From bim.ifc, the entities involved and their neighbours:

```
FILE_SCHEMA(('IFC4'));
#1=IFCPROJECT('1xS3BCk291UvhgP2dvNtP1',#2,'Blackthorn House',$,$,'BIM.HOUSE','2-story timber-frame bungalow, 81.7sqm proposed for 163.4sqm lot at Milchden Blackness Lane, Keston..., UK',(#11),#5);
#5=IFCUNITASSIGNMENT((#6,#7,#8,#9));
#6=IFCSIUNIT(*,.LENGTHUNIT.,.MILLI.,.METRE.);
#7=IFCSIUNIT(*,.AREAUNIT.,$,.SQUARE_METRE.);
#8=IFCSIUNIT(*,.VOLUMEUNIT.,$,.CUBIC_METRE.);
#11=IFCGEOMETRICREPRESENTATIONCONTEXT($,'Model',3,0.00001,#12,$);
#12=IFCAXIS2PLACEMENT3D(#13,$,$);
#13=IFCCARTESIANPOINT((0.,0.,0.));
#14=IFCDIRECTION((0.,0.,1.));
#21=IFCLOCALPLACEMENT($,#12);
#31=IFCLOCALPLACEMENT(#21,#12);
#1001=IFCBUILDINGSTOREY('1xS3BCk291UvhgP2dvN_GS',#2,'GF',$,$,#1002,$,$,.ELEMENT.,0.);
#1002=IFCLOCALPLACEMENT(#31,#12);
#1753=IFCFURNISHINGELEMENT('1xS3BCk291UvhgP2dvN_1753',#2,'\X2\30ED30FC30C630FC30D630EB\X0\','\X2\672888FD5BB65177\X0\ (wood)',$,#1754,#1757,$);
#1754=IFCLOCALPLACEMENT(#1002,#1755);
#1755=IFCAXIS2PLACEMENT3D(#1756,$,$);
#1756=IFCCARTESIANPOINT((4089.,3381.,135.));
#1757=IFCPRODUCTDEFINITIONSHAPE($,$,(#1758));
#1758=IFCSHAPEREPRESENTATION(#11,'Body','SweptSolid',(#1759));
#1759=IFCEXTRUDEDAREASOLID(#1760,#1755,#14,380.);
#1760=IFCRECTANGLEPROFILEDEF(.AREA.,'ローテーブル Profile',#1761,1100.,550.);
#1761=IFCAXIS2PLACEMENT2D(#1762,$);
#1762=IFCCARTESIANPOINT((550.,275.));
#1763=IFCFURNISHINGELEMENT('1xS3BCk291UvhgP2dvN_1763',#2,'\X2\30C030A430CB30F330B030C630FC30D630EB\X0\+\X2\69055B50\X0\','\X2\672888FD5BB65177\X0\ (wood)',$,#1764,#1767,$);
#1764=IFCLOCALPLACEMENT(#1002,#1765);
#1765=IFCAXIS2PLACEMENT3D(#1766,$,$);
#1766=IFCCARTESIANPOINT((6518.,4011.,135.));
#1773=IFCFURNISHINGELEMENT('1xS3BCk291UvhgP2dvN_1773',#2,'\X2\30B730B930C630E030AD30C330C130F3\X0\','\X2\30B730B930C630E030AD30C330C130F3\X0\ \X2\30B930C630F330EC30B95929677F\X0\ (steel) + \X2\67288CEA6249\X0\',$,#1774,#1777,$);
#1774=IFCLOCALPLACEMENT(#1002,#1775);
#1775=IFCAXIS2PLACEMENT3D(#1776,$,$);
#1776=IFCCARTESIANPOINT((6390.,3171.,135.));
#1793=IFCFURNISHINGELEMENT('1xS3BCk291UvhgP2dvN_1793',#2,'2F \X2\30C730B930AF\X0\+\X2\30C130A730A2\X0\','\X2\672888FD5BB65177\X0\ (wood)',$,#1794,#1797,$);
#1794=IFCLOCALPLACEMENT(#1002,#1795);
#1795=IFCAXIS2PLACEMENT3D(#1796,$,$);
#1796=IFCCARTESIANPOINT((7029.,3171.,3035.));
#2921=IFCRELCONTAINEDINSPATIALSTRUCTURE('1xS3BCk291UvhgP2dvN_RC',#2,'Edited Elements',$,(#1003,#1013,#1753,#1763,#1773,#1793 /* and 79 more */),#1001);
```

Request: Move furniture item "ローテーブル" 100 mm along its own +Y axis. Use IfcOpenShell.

```python
import ifcopenshell
import ifcopenshell.api.geometry
import ifcopenshell.util.placement

model = ifcopenshell.open("bim.ifc")

item = model.by_guid("1xS3BCk291UvhgP2dvN_1753")
matrix = ifcopenshell.util.placement.get_local_placement(item.ObjectPlacement)
matrix[:3, 3] += matrix[:3, 1] * 100.0
ifcopenshell.api.geometry.edit_object_placement(model, product=item, matrix=matrix, is_si=False)

print(ifcopenshell.util.placement.get_local_placement(item.ObjectPlacement).round(3) + 0.0)

model.write("bim_updated.ifc")
```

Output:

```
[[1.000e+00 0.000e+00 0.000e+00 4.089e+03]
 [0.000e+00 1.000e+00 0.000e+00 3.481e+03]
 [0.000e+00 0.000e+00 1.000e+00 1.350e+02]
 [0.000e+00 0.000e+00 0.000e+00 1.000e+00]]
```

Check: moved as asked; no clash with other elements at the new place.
